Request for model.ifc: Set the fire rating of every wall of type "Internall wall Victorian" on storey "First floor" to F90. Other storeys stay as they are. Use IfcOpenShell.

First a look at what the model holds.

```python
import ifcopenshell
import ifcopenshell.util.element

model = ifcopenshell.open("model.ifc")
print(model.schema)
storey = next(s for s in model.by_type("IfcBuildingStorey") if s.Name == "First floor")
walls = [e for e in ifcopenshell.util.element.get_decomposition(storey) if e.is_a("IfcWall")]
seen = {}
for e in walls:
    element_type = ifcopenshell.util.element.get_type(e)
    key = (element_type.Name if element_type != e and element_type else None, ifcopenshell.util.element.get_pset(e, "Pset_WallCommon", "FireRating"))
    seen[key] = seen.get(key, 0) + 1
for (name, value), count in sorted(seen.items(), key=str):
    print(count, "x", name, "|", value)
```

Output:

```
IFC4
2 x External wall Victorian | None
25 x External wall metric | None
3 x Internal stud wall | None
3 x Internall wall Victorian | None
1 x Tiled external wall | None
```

```python
import ifcopenshell
import ifcopenshell.api.pset
import ifcopenshell.util.element

model = ifcopenshell.open("model.ifc")

storey = next(s for s in model.by_type("IfcBuildingStorey") if s.Name == "First floor")
walls = [e for e in ifcopenshell.util.element.get_decomposition(storey) if e.is_a("IfcWall")]

count = 0
for e in walls:
    element_type = ifcopenshell.util.element.get_type(e)
    if element_type in (None, e) or element_type.Name != "Internall wall Victorian":
        continue
    # add_pset returns the element's existing set when there is one.
    pset = ifcopenshell.api.pset.add_pset(model, product=e, name="Pset_WallCommon")
    ifcopenshell.api.pset.edit_pset(model, pset=pset, properties={"FireRating": "F90"})
    count += 1

print(count, "walls updated")

model.write("model_v2.ifc")
```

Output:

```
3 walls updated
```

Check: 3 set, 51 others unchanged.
